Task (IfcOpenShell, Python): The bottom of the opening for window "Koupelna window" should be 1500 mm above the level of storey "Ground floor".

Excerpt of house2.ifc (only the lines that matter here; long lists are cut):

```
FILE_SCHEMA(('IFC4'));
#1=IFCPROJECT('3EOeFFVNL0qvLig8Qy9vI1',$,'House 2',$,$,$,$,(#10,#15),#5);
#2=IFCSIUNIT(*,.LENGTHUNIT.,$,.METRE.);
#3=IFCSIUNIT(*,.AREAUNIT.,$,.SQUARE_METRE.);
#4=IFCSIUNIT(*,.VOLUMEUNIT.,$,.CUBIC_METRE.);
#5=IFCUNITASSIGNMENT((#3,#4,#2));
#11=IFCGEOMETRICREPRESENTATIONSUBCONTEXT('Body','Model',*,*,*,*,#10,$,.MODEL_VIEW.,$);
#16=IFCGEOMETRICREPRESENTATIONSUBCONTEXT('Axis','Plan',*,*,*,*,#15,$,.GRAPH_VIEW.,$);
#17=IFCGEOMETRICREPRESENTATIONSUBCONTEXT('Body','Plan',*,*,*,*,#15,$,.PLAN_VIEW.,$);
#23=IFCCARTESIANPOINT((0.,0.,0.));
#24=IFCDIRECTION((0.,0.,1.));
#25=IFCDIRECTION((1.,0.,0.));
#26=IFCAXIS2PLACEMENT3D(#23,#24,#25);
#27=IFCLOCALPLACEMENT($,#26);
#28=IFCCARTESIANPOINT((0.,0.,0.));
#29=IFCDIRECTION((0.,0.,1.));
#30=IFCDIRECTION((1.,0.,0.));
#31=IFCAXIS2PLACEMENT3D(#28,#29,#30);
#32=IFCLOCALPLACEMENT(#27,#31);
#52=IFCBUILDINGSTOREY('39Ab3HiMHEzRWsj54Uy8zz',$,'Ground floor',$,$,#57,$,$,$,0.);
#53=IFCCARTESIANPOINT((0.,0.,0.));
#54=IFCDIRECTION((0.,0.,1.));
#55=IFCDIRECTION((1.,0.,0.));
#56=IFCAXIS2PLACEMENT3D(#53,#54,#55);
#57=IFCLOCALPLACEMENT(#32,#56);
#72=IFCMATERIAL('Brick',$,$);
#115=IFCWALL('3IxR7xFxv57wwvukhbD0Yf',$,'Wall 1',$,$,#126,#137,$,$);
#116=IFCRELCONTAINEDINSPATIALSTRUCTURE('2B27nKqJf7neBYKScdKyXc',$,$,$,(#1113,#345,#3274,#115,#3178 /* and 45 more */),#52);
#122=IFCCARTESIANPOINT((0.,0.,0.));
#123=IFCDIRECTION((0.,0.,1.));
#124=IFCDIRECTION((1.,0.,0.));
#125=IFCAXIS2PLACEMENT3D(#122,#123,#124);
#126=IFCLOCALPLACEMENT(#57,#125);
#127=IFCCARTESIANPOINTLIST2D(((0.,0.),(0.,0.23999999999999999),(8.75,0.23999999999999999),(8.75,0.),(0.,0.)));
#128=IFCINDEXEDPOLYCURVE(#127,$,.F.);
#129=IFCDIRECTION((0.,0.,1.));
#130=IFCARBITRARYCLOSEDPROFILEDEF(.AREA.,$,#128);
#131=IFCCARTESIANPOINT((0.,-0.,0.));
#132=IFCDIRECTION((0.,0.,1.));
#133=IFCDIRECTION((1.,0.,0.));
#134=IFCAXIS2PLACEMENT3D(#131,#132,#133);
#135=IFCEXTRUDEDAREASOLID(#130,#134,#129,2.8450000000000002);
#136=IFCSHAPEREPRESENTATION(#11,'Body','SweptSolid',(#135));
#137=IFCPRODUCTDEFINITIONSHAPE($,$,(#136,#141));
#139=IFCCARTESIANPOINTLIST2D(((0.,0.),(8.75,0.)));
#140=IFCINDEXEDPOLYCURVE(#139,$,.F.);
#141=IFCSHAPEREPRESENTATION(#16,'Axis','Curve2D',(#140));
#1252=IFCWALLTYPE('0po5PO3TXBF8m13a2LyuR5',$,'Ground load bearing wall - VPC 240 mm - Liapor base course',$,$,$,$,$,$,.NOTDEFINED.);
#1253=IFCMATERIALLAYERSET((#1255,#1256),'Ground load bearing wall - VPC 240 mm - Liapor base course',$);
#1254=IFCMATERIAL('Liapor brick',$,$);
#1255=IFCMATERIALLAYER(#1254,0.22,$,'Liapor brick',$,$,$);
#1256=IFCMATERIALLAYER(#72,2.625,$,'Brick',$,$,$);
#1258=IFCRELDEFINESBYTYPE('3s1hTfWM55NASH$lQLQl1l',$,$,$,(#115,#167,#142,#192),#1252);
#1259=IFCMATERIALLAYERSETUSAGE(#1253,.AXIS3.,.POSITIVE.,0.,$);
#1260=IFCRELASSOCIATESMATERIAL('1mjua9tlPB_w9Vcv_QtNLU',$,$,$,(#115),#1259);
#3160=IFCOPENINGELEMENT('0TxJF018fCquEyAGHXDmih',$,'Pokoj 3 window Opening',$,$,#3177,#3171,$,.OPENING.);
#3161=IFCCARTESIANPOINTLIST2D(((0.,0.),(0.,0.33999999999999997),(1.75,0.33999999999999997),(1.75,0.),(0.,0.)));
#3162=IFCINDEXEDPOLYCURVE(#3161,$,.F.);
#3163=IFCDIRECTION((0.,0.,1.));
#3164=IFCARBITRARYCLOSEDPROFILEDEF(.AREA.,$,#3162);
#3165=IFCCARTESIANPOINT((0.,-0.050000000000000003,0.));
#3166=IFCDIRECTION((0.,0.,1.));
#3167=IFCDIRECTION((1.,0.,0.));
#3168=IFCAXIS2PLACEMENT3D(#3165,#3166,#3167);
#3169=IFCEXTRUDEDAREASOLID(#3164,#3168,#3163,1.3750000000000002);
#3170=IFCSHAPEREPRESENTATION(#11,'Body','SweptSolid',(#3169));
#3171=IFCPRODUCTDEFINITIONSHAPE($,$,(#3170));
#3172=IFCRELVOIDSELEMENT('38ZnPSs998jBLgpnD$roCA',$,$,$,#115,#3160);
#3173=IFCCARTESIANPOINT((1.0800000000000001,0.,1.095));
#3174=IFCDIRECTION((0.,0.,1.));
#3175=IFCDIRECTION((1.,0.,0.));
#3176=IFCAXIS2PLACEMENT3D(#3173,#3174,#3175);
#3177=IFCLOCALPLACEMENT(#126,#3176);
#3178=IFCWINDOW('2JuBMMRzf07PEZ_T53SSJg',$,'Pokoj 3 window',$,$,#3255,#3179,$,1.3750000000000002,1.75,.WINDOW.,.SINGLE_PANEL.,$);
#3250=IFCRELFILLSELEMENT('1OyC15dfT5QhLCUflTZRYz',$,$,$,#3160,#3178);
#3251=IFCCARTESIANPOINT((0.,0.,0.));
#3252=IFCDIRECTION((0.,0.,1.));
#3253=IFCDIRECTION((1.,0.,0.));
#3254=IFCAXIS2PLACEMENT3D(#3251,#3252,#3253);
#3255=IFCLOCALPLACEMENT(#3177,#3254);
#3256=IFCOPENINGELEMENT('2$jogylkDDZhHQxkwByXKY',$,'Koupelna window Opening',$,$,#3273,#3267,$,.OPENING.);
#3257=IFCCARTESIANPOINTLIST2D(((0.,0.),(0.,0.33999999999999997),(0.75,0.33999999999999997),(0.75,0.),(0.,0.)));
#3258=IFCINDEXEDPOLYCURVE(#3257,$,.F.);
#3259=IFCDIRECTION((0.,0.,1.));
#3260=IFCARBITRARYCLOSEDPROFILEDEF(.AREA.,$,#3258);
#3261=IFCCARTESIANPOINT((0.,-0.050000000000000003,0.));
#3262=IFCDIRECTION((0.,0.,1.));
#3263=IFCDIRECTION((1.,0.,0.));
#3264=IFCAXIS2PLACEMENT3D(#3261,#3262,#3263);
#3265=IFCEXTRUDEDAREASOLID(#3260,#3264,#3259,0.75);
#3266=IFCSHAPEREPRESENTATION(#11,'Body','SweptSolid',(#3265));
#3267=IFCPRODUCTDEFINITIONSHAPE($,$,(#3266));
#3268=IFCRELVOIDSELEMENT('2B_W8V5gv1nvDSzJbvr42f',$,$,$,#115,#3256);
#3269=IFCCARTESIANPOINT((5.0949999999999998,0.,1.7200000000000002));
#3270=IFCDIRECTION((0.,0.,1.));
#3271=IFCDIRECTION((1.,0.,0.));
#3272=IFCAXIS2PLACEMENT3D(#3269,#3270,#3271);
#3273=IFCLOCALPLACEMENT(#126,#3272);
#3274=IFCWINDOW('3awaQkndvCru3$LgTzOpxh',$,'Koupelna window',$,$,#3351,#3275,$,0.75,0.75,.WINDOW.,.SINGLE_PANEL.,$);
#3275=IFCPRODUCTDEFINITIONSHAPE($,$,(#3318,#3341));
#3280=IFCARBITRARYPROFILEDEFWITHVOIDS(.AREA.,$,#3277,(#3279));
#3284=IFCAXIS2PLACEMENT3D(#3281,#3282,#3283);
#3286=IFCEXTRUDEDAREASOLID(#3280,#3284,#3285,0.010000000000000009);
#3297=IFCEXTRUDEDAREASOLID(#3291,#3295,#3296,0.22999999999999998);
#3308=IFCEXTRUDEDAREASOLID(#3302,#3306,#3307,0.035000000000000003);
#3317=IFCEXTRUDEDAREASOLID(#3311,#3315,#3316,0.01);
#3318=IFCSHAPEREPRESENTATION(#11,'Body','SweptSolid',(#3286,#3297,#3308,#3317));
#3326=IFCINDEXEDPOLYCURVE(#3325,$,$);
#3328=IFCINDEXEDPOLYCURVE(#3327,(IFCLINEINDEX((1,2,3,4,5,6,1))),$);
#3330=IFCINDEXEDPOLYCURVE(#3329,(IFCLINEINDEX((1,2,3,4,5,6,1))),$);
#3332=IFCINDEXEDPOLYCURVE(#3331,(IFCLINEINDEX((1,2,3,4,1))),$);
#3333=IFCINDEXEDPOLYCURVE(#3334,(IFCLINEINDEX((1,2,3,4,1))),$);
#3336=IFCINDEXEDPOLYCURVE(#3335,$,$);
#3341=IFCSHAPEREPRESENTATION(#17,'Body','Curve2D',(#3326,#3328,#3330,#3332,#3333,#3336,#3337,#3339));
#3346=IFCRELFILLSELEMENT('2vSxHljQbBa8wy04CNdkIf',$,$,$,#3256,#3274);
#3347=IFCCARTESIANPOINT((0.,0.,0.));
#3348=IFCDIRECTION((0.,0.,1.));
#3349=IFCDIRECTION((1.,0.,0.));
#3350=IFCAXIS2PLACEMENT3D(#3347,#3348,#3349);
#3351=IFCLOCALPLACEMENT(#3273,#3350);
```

```python
import numpy as np
import ifcopenshell
import ifcopenshell.api.geometry
import ifcopenshell.geom
import ifcopenshell.util.element
import ifcopenshell.util.placement
import ifcopenshell.util.shape
import ifcopenshell.util.unit

model = ifcopenshell.open("house2.ifc")
unit_scale = ifcopenshell.util.unit.calculate_unit_scale(model)

window = model.by_guid("3awaQkndvCru3$LgTzOpxh")
opening = window.FillsVoids[0].RelatingOpeningElement
storey = ifcopenshell.util.element.get_container(window, ifc_class="IfcBuildingStorey")
level = ifcopenshell.util.placement.get_local_placement(storey.ObjectPlacement)[2, 3]

# The opening's origin need not be at the sill, so measure its lowest point.
shape = ifcopenshell.geom.create_shape(ifcopenshell.geom.settings(), opening)
bottom = ifcopenshell.util.shape.get_shape_bottom_elevation(shape, shape.geometry) / unit_scale
dz = level + 1.5 - bottom

shift = np.array([0.0, 0.0, dz])
# The window is placed relative to its opening, so it follows when the opening moves.
matrix = ifcopenshell.util.placement.get_local_placement(opening.ObjectPlacement)
matrix[:3, 3] += shift
ifcopenshell.api.geometry.edit_object_placement(
    model, product=opening, matrix=matrix, is_si=False, should_transform_children=True
)

print(f"moved by {dz * unit_scale:+.3f} m")

model.write("house2_rev.ifc")
```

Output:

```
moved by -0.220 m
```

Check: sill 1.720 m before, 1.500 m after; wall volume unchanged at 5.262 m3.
